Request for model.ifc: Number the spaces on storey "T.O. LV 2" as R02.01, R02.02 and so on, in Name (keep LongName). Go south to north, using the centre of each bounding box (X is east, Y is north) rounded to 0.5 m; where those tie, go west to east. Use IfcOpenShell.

First a look at what the model holds.

```python
import ifcopenshell
import ifcopenshell.util.element
import ifcopenshell.util.placement

model = ifcopenshell.open("model.ifc")
print(model.schema)
storey = next(s for s in model.by_type("IfcBuildingStorey") if s.Name == "T.O. LV 2")
spaces = [e for e in ifcopenshell.util.element.get_decomposition(storey) if e.is_a("IfcSpace")]
for e in sorted(spaces, key=lambda e: e.id()):
    origin = ifcopenshell.util.placement.get_local_placement(e.ObjectPlacement)[:3, 3]
    print(e.id(), e.Name, e.LongName, origin.round(2) + 0.0, sep=" | ")
```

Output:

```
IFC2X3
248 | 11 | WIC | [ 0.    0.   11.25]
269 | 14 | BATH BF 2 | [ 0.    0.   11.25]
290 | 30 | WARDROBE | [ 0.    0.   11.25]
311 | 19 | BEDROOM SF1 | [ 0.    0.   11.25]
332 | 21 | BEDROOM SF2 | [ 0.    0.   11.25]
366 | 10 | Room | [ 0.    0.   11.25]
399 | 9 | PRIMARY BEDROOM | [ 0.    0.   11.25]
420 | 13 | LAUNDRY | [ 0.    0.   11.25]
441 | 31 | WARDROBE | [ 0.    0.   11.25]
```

```python
import ifcopenshell
import ifcopenshell.geom
import ifcopenshell.util.element
import ifcopenshell.util.shape

model = ifcopenshell.open("model.ifc")
settings = ifcopenshell.geom.settings()
settings.set("use-world-coords", True)


def centre(element):
    shape = ifcopenshell.geom.create_shape(settings, element)
    return ifcopenshell.util.shape.get_bbox_centroid(shape.geometry)


storey = next(s for s in model.by_type("IfcBuildingStorey") if s.Name == "T.O. LV 2")
spaces = [e for e in ifcopenshell.util.element.get_decomposition(storey) if e.is_a("IfcSpace")]

# Insertion points can sit at a corner or the storey origin, so sort by the geometry (in metres).
centres = {e: centre(e) for e in spaces}
spaces.sort(key=lambda e: (round(centres[e][1] / 0.5), centres[e][0]))

for i, e in enumerate(spaces, start=1):
    number = f"R02.{i:02d}"
    e.Name = number
    print(e.id(), number)

model.write("model_updated.ifc")
```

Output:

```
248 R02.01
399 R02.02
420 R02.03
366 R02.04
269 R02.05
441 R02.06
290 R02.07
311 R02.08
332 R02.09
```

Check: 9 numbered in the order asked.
